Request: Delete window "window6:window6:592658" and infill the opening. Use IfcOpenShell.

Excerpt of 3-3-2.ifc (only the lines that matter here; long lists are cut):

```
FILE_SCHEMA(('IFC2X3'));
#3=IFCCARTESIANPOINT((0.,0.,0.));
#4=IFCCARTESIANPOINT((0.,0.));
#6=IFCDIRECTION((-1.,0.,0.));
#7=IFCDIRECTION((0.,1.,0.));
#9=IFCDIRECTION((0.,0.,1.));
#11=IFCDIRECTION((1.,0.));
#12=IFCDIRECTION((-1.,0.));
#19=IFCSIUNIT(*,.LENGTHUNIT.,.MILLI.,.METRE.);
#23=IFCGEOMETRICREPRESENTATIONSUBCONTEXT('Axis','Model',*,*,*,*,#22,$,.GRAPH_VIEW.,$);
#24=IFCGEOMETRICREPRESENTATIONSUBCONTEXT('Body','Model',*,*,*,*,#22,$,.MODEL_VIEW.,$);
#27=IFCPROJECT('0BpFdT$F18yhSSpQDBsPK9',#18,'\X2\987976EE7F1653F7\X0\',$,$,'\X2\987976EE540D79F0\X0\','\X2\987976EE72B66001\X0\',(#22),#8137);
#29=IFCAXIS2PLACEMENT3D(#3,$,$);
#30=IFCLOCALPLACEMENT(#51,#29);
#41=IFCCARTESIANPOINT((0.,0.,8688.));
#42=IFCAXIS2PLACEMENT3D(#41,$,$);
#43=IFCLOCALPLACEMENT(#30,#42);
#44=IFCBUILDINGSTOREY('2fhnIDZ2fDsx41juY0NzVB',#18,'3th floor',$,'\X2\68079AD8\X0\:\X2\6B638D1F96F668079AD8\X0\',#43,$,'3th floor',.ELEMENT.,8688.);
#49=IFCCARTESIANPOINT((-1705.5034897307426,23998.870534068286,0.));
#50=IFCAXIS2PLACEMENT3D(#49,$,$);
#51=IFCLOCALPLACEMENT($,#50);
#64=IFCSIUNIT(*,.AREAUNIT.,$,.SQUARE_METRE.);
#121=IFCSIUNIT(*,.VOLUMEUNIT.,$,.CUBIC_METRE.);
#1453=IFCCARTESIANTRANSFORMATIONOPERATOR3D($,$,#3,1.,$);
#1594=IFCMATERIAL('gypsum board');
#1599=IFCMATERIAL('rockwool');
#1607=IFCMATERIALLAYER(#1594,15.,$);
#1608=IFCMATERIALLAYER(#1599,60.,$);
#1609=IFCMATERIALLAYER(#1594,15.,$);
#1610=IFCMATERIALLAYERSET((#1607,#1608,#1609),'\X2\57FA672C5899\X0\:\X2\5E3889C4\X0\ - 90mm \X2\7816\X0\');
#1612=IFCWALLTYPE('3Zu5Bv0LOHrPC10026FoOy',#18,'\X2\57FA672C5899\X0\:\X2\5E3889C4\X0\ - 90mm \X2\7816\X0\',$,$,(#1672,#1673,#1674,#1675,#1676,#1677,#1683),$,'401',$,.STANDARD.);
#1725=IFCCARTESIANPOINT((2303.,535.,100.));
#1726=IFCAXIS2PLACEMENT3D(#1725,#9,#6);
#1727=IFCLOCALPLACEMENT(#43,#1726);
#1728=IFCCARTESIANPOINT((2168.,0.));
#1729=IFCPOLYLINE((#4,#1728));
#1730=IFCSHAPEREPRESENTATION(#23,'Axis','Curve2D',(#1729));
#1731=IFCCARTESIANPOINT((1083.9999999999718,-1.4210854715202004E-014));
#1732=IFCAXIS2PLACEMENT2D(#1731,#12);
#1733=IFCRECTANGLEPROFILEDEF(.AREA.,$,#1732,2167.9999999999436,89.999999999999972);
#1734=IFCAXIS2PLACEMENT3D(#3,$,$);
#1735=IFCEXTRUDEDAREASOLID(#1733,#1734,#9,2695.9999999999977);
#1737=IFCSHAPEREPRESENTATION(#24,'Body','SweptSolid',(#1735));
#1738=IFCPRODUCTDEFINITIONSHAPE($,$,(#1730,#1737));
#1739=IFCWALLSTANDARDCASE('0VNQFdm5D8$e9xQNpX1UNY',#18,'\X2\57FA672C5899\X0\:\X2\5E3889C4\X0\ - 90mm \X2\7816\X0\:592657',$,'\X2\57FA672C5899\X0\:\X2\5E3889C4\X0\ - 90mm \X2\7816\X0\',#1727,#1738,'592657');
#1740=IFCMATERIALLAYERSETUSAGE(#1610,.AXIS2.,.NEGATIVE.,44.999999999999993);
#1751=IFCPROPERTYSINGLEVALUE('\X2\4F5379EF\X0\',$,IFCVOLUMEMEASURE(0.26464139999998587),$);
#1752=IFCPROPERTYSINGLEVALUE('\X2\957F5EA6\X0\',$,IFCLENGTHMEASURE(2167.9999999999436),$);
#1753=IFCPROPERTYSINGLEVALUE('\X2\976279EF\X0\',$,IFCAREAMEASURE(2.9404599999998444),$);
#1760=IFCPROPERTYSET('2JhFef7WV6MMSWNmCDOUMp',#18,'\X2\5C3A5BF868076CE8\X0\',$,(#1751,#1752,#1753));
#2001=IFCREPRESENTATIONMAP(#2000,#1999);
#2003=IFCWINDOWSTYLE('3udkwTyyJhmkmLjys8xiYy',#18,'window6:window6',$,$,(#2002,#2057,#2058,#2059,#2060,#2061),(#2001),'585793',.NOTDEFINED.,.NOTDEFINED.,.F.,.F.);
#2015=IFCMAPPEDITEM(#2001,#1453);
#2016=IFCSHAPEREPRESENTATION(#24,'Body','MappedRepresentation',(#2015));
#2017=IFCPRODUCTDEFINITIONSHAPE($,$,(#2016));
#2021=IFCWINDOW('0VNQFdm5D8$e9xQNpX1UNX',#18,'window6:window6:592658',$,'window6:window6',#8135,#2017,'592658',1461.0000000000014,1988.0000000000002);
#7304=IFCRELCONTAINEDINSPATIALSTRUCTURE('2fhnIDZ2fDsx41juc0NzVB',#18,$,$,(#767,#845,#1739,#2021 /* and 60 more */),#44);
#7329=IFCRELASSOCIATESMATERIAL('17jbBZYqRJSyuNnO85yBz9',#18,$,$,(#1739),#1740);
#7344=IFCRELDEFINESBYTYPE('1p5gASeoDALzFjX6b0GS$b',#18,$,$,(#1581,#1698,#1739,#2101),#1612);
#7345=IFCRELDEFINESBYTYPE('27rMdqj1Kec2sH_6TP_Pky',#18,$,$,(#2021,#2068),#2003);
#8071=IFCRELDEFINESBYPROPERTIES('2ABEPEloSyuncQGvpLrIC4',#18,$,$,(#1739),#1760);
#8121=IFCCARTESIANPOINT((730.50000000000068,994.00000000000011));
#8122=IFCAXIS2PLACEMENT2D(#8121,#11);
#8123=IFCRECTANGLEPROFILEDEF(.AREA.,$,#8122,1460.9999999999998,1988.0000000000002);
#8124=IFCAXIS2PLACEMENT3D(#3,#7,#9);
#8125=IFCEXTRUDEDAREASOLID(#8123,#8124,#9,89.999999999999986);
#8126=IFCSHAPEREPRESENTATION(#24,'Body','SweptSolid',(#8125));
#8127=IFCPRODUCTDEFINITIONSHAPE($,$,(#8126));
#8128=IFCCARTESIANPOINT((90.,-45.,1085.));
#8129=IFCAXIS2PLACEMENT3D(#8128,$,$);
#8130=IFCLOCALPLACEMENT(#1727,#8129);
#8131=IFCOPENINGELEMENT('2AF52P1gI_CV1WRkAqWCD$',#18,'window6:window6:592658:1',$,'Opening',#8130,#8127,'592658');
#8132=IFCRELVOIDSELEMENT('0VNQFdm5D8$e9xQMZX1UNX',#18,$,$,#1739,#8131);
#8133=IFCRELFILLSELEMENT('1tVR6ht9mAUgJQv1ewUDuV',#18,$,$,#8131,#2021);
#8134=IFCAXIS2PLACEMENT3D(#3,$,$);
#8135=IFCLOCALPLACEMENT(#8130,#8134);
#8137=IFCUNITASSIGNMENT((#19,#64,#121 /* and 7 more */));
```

```python
import ifcopenshell
import ifcopenshell.api.feature
import ifcopenshell.api.pset
import ifcopenshell.api.root
import ifcopenshell.geom
import ifcopenshell.util.element
import ifcopenshell.util.shape
import ifcopenshell.util.unit

model = ifcopenshell.open("3-3-2.ifc")
area_scale = ifcopenshell.util.unit.calculate_unit_scale(model, "AREAUNIT")
volume_scale = ifcopenshell.util.unit.calculate_unit_scale(model, "VOLUMEUNIT")
settings = ifcopenshell.geom.settings()


def volume(element):
    """Net volume in cubic metres, openings subtracted."""
    shape = ifcopenshell.geom.create_shape(settings, element)
    return ifcopenshell.util.shape.get_volume(shape.geometry)


window = model.by_id(2021)
opening = window.FillsVoids[0].RelatingOpeningElement
wall = opening.VoidsElements[0].RelatingBuildingElement
before = volume(wall)

ifcopenshell.api.root.remove_product(model, product=window)
ifcopenshell.api.feature.remove_feature(model, feature=opening)

after = volume(wall)
thickness = 0.09  # wall thickness in metres

# Update the wall's stored quantities.
pset = model.by_id(ifcopenshell.util.element.get_pset(wall, "尺寸标注", should_inherit=False)["id"])
ifcopenshell.api.pset.edit_pset(model, pset=pset, properties={
    "体积": model.create_entity("IfcVolumeMeasure", after / volume_scale),
    "面积": model.create_entity("IfcAreaMeasure", after / thickness / area_scale),
})

print(f"wall volume {before:.3f} -> {after:.3f} m3")

model.write("3-3-2-out.ifc")
```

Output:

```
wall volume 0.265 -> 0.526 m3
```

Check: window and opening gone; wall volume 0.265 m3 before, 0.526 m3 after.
